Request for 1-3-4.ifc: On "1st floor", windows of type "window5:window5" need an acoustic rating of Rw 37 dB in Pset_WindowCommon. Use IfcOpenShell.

First a look at what the model holds.

```python
import ifcopenshell
import ifcopenshell.util.element

model = ifcopenshell.open("1-3-4.ifc")
print(model.schema)
storey = next(s for s in model.by_type("IfcBuildingStorey") if s.Name == "1st floor")
windows = [e for e in ifcopenshell.util.element.get_decomposition(storey) if e.is_a("IfcWindow")]
seen = {}
for e in windows:
    element_type = ifcopenshell.util.element.get_type(e)
    key = (element_type.Name if element_type != e and element_type else None, ifcopenshell.util.element.get_pset(e, "Pset_WindowCommon", "AcousticRating"))
    seen[key] = seen.get(key, 0) + 1
for (name, value), count in sorted(seen.items(), key=str):
    print(count, "x", name, "|", value)
```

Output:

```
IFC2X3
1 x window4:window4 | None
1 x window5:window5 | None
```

```python
import ifcopenshell
import ifcopenshell.api.pset
import ifcopenshell.util.element

model = ifcopenshell.open("1-3-4.ifc")

storey = next(s for s in model.by_type("IfcBuildingStorey") if s.Name == "1st floor")
windows = [e for e in ifcopenshell.util.element.get_decomposition(storey) if e.is_a("IfcWindow")]

count = 0
for e in windows:
    element_type = ifcopenshell.util.element.get_type(e)
    if element_type in (None, e) or element_type.Name != "window5:window5":
        continue
    # add_pset returns the element's existing set when there is one.
    pset = ifcopenshell.api.pset.add_pset(model, product=e, name="Pset_WindowCommon")
    ifcopenshell.api.pset.edit_pset(model, pset=pset, properties={"AcousticRating": "Rw 37 dB"})
    count += 1

print(count, "windows updated")

model.write("1-3-4_updated.ifc")
```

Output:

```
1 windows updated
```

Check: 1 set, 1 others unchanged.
